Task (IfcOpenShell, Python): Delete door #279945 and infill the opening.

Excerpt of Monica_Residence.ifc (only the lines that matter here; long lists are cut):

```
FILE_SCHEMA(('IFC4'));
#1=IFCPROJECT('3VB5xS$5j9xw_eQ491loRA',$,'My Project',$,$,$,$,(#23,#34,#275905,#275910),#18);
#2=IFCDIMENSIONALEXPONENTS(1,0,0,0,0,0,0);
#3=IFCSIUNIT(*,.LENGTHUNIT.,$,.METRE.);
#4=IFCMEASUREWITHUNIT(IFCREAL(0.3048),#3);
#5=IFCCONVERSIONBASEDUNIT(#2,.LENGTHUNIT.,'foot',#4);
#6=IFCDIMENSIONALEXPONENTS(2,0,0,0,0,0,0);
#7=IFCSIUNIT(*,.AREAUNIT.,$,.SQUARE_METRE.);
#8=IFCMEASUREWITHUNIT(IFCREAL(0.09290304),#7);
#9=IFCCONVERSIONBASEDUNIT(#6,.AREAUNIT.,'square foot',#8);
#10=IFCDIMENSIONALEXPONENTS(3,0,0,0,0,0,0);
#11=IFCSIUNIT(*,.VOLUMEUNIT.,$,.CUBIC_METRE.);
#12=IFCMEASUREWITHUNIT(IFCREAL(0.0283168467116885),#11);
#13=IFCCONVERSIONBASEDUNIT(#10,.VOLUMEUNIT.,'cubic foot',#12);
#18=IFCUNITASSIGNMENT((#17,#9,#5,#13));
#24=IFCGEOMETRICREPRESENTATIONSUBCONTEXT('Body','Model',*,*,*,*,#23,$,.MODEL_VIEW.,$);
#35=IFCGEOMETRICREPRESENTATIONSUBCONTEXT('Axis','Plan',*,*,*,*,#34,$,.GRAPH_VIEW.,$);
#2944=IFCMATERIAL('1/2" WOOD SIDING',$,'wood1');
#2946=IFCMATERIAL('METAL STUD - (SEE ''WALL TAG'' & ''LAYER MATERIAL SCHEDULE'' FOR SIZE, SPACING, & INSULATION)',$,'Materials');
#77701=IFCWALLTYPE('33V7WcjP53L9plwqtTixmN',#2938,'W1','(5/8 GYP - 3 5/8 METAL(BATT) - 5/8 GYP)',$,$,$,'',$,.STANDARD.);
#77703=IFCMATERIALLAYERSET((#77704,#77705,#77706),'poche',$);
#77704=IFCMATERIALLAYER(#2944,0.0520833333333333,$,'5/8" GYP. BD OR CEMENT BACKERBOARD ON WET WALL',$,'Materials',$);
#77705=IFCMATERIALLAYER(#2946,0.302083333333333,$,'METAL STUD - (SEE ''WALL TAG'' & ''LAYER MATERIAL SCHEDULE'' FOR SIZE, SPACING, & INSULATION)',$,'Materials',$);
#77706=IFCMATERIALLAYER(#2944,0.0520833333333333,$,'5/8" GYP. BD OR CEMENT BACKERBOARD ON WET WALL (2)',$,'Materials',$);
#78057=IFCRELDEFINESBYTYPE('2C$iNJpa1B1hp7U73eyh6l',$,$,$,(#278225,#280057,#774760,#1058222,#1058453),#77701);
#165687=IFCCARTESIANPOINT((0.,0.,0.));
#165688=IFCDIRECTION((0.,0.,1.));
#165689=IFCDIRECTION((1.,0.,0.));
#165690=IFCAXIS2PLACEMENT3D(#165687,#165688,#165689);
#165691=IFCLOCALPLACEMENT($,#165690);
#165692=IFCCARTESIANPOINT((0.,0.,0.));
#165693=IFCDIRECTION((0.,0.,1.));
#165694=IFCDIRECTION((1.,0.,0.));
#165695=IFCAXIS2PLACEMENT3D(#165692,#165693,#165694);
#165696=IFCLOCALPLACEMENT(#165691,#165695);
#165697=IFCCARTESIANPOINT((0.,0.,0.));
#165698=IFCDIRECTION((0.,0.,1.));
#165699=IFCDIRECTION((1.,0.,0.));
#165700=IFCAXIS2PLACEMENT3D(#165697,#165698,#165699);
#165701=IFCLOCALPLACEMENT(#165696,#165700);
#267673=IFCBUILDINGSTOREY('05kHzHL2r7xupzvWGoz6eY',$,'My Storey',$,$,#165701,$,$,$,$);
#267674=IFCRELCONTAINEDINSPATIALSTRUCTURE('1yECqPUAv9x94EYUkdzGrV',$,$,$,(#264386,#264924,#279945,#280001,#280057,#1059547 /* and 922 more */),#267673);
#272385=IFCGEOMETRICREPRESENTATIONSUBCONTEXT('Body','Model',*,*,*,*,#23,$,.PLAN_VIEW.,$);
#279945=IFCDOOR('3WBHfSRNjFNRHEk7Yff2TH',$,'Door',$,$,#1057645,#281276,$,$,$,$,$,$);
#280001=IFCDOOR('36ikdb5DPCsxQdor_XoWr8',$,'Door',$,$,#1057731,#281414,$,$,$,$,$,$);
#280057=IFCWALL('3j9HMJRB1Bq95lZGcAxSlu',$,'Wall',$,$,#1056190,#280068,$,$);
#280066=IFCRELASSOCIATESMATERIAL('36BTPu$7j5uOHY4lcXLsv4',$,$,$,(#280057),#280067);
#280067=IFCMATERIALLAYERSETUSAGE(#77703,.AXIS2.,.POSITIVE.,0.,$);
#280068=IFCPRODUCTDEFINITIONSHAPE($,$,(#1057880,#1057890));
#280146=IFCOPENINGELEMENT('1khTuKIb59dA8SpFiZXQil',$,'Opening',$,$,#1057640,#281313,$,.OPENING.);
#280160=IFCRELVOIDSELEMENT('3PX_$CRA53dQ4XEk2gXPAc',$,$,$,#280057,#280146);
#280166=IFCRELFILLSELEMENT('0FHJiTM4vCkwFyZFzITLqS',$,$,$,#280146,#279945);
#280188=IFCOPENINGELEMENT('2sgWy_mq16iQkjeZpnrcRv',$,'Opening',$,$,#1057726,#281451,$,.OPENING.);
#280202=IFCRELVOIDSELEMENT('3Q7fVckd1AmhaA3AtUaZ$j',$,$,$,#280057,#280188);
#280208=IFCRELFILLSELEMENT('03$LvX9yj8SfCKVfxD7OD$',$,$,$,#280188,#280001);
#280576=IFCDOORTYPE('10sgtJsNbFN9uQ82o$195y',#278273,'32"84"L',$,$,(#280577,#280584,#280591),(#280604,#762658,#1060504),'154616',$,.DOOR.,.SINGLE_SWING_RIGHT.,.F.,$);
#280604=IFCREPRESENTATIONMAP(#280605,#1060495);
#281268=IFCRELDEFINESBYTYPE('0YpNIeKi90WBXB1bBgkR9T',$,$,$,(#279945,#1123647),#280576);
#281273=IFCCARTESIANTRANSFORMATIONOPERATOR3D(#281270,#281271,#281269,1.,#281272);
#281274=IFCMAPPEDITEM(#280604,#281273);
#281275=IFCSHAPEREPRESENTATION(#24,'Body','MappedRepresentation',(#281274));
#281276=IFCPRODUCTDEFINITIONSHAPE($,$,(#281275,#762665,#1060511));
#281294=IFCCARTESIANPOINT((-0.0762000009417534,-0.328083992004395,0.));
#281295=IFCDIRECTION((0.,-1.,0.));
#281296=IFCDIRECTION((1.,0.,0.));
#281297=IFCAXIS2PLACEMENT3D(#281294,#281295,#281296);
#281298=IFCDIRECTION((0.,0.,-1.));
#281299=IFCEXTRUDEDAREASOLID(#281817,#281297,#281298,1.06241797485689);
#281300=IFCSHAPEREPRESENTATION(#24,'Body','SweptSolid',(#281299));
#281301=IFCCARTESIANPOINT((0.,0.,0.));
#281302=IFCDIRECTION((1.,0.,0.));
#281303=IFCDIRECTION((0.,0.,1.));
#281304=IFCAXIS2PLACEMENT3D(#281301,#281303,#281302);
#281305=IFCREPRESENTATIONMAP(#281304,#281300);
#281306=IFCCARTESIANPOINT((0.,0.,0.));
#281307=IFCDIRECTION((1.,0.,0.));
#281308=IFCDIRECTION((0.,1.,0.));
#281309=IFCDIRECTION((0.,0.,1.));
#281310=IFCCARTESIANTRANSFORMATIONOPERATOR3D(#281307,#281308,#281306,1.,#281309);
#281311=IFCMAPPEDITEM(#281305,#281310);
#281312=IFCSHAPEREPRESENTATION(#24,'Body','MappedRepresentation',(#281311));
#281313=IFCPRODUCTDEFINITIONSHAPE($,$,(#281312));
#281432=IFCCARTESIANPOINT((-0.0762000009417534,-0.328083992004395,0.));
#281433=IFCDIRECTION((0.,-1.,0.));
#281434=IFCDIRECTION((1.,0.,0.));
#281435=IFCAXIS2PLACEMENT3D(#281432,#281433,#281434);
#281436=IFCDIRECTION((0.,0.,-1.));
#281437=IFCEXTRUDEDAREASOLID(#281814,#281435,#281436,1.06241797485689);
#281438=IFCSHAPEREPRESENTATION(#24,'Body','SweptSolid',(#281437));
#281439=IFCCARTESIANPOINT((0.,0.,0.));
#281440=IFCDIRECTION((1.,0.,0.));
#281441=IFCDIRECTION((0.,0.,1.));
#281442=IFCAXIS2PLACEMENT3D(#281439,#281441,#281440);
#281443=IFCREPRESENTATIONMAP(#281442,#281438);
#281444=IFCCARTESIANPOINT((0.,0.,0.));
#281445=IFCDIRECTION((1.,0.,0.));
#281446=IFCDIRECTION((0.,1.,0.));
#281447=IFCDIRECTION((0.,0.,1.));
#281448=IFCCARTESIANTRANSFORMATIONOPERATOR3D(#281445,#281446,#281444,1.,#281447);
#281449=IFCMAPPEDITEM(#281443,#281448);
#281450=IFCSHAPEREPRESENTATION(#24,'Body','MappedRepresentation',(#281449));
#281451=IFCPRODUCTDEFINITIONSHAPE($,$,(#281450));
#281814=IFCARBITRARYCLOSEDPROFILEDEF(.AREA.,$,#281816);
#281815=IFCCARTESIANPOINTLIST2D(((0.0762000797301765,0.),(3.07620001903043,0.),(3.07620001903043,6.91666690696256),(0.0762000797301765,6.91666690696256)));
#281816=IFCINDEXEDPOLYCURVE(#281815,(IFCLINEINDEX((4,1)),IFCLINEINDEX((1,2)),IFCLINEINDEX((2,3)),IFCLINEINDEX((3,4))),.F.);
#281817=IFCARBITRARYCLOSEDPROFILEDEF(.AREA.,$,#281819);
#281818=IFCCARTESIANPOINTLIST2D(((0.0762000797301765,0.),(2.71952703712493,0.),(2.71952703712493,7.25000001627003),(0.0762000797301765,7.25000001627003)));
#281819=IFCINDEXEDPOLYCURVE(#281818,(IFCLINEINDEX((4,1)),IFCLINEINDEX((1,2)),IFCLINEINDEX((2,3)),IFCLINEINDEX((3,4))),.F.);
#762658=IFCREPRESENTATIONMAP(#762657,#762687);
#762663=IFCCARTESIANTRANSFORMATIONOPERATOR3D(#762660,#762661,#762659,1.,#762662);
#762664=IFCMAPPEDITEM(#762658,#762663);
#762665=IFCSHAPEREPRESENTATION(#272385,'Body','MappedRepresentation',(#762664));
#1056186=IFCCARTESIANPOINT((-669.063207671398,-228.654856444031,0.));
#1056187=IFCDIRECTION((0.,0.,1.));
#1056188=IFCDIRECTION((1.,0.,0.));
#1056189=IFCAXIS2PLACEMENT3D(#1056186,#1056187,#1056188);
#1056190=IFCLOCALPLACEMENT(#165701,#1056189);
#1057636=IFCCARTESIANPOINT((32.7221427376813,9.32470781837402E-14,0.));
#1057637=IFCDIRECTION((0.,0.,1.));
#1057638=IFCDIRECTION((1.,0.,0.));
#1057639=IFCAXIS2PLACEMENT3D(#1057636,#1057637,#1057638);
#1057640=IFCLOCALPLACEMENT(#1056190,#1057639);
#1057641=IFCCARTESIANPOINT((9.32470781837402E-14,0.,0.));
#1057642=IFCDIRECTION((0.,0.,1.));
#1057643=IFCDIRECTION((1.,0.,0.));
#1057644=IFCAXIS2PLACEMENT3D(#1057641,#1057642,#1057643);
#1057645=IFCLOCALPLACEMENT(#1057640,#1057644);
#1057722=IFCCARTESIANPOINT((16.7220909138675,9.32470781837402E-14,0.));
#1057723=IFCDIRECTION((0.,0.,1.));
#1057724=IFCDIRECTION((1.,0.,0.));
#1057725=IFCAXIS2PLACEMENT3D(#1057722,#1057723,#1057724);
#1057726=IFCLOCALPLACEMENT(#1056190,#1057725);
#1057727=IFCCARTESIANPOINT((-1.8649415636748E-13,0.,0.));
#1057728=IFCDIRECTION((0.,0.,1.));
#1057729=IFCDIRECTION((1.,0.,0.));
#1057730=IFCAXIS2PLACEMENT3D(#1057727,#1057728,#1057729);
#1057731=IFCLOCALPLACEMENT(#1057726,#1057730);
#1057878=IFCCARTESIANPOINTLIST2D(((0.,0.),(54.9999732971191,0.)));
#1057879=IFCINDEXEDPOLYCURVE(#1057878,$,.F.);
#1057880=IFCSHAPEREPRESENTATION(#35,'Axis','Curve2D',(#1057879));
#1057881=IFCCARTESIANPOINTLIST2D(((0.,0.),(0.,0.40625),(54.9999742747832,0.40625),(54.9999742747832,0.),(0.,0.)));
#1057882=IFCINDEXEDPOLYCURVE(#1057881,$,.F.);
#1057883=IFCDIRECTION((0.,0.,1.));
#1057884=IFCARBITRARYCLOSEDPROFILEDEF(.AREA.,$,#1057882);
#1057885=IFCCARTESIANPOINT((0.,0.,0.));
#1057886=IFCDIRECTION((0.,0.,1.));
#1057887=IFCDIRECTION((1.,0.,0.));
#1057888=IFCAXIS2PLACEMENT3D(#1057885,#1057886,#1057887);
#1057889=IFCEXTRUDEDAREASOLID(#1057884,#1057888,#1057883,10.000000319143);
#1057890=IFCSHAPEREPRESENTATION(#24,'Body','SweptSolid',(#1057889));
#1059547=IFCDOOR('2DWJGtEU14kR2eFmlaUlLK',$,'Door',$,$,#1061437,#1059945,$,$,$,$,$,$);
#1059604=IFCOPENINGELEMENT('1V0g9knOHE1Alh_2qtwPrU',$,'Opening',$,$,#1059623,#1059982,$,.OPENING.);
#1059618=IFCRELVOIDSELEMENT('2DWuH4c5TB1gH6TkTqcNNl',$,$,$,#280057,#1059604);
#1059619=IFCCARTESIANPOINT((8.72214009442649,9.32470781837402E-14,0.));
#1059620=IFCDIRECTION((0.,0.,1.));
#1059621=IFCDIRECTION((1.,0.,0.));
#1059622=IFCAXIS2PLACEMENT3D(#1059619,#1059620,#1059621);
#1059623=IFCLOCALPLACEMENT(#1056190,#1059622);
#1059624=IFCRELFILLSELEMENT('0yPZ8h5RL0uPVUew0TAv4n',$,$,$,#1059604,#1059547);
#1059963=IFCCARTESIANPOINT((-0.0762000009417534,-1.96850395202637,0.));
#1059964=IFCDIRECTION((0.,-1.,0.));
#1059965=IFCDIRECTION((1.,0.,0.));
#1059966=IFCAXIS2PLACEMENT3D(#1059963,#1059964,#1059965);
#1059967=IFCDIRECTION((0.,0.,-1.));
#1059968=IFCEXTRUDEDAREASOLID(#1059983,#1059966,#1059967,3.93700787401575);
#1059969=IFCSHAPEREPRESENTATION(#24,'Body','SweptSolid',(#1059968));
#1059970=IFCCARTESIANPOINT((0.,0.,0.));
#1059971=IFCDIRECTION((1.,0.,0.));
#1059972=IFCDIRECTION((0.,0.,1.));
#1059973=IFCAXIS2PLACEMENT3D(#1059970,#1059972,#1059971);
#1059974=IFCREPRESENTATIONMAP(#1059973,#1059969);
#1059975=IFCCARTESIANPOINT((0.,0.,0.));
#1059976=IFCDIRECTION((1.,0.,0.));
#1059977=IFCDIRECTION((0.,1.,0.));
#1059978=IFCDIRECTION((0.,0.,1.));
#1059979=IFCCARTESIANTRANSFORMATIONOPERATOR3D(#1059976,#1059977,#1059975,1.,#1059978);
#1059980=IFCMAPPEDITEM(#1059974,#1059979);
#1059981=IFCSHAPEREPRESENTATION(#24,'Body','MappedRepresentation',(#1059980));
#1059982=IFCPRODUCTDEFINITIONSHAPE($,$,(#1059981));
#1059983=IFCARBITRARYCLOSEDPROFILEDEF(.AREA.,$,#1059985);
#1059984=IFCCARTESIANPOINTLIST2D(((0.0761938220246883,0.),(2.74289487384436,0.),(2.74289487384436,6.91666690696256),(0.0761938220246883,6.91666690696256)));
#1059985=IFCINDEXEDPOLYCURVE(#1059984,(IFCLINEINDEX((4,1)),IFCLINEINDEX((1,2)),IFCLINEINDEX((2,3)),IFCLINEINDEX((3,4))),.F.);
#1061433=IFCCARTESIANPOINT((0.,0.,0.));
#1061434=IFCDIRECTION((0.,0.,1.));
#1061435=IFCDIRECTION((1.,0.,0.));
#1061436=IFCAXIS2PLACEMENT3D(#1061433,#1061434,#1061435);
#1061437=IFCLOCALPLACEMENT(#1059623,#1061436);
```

```python
import ifcopenshell
import ifcopenshell.api.feature
import ifcopenshell.api.root
import ifcopenshell.geom
import ifcopenshell.util.shape

model = ifcopenshell.open("Monica_Residence.ifc")
settings = ifcopenshell.geom.settings()


def volume(element):
    """Net volume in cubic metres, openings subtracted."""
    shape = ifcopenshell.geom.create_shape(settings, element)
    return ifcopenshell.util.shape.get_volume(shape.geometry)


door = model.by_id(279945)
opening = door.FillsVoids[0].RelatingOpeningElement
wall = opening.VoidsElements[0].RelatingBuildingElement
before = volume(wall)

ifcopenshell.api.root.remove_product(model, product=door)
ifcopenshell.api.feature.remove_feature(model, feature=opening)

after = volume(wall)

print(f"wall volume {before:.3f} -> {after:.3f} m3")

model.write("Monica_Residence_rev.ifc")
```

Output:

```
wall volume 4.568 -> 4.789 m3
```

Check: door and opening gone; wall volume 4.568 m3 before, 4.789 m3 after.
